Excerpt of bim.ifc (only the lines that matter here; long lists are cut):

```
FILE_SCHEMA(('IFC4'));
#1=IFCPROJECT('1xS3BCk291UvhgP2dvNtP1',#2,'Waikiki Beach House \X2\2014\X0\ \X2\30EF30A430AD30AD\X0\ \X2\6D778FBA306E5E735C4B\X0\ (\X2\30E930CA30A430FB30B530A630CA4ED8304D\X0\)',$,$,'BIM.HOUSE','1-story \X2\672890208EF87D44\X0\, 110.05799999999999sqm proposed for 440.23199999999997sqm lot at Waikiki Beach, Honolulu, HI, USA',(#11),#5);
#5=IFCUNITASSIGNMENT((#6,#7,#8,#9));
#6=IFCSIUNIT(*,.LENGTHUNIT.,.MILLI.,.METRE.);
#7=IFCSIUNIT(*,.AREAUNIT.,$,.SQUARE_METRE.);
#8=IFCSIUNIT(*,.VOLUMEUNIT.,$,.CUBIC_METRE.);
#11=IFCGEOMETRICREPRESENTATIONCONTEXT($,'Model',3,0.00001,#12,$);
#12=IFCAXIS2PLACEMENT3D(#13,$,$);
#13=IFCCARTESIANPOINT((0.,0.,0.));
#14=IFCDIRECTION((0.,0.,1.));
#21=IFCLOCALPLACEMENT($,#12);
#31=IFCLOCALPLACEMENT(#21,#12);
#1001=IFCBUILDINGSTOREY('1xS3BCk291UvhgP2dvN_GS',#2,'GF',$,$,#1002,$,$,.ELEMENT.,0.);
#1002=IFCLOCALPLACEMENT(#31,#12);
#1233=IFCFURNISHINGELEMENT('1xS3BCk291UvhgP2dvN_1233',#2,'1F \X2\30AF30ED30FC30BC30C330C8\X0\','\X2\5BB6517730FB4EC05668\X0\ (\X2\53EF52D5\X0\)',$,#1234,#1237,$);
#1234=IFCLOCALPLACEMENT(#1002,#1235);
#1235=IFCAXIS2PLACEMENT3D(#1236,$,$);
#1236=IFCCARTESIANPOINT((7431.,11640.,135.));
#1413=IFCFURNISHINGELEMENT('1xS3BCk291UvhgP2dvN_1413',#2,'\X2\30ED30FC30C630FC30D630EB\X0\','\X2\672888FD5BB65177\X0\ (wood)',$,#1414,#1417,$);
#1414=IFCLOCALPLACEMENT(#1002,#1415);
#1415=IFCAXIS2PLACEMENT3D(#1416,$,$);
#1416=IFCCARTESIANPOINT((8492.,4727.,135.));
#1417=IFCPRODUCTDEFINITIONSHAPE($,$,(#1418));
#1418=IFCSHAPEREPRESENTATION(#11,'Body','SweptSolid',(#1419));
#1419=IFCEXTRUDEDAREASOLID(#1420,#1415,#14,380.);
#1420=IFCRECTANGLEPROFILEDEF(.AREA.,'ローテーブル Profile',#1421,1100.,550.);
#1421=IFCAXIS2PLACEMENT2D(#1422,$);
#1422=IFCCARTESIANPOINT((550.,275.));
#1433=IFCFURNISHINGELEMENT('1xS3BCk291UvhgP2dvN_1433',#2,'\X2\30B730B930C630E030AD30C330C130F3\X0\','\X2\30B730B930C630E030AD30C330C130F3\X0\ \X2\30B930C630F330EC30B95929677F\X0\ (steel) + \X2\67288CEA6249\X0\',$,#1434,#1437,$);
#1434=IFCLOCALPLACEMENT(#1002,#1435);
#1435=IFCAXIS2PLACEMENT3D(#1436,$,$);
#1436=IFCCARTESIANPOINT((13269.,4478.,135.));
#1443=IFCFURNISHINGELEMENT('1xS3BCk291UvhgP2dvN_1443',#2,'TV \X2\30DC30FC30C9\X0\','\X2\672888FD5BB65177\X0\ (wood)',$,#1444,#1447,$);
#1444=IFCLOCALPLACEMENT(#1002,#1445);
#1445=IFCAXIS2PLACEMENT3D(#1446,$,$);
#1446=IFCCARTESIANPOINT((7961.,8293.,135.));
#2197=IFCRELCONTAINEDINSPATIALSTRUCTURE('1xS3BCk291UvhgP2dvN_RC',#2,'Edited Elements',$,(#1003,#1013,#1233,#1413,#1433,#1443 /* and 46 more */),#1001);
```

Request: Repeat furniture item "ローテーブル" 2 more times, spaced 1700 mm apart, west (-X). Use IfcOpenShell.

```python
import numpy as np
import ifcopenshell
import ifcopenshell.api.geometry
import ifcopenshell.api.root
import ifcopenshell.util.element
import ifcopenshell.util.placement
import ifcopenshell.util.unit

model = ifcopenshell.open("bim.ifc")
unit_scale = ifcopenshell.util.unit.calculate_unit_scale(model)


def reuse_history(source, copy):
    """copy_class also copies each property set's owner history, people and application; keep the originals."""
    for rel in copy.IsDefinedBy:
        if rel.is_a("IfcRelDefinesByProperties") and (history := rel.RelatingPropertyDefinition.OwnerHistory):
            rel.RelatingPropertyDefinition.OwnerHistory = source.OwnerHistory
            ifcopenshell.util.element.remove_deep2(model, history)


source = model.by_guid("1xS3BCk291UvhgP2dvN_1413")
base = ifcopenshell.util.placement.get_local_placement(source.ObjectPlacement)
step = np.array([-1.0, 0.0, 0.0]) * 1.7 / unit_scale

for i in range(1, 3):
    copy = ifcopenshell.api.root.copy_class(model, product=source)
    copy.Representation = ifcopenshell.util.element.copy_deep(
        model, source.Representation, exclude=["IfcGeometricRepresentationContext", "IfcRepresentationMap"]
    )
    reuse_history(source, copy)
    matrix = base.copy()
    matrix[:3, 3] += i * step
    print("added at", matrix[:3, 3].round(3) + 0.0)
    ifcopenshell.api.geometry.edit_object_placement(model, product=copy, matrix=matrix, is_si=False)

model.write("bim-out.ifc")
```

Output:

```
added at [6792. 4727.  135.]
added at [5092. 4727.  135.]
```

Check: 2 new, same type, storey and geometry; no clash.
